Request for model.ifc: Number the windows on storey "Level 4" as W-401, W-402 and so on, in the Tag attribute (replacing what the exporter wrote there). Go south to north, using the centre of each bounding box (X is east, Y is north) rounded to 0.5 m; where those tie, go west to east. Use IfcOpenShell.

First a look at what the model holds.

```python
import ifcopenshell
import ifcopenshell.util.element
import ifcopenshell.util.placement

model = ifcopenshell.open("model.ifc")
print(model.schema)
storey = next(s for s in model.by_type("IfcBuildingStorey") if s.Name == "Level 4")
windows = [e for e in ifcopenshell.util.element.get_decomposition(storey) if e.is_a("IfcWindow")]
for e in sorted(windows, key=lambda e: e.id()):
    origin = ifcopenshell.util.placement.get_local_placement(e.ObjectPlacement)[:3, 3]
    print(e.id(), e.Tag, e.Name, origin.round(2) + 0.0, sep=" | ")
```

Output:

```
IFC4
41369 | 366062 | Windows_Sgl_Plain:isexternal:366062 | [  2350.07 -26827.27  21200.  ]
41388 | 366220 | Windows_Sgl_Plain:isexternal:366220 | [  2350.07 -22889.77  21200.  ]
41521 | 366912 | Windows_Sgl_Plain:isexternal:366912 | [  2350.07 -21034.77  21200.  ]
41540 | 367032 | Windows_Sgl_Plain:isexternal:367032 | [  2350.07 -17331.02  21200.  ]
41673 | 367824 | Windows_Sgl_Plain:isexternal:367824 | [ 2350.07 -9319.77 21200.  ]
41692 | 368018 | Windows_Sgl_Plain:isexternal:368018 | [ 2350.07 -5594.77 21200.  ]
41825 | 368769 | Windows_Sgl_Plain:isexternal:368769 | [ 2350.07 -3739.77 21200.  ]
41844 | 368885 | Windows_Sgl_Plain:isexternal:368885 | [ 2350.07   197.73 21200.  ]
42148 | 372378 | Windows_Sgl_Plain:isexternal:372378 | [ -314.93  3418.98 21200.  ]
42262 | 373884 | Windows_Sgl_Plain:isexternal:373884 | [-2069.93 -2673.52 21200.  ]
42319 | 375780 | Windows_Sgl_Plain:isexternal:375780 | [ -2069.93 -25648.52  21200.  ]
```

```python
import ifcopenshell
import ifcopenshell.geom
import ifcopenshell.util.element
import ifcopenshell.util.shape

model = ifcopenshell.open("model.ifc")
settings = ifcopenshell.geom.settings()
settings.set("use-world-coords", True)


def centre(element):
    shape = ifcopenshell.geom.create_shape(settings, element)
    return ifcopenshell.util.shape.get_bbox_centroid(shape.geometry)


storey = next(s for s in model.by_type("IfcBuildingStorey") if s.Name == "Level 4")
windows = [e for e in ifcopenshell.util.element.get_decomposition(storey) if e.is_a("IfcWindow")]

# Insertion points can sit at a corner or the storey origin, so sort by the geometry (in metres).
centres = {e: centre(e) for e in windows}
windows.sort(key=lambda e: (round(centres[e][1] / 0.5), centres[e][0]))

for i, e in enumerate(windows, start=1):
    number = f"W-4{i:02d}"
    e.Tag = number
    print(e.id(), number)

model.write("model-out.ifc")
```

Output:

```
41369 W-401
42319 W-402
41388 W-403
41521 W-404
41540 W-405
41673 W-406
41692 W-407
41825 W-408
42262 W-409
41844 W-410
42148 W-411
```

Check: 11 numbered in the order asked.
